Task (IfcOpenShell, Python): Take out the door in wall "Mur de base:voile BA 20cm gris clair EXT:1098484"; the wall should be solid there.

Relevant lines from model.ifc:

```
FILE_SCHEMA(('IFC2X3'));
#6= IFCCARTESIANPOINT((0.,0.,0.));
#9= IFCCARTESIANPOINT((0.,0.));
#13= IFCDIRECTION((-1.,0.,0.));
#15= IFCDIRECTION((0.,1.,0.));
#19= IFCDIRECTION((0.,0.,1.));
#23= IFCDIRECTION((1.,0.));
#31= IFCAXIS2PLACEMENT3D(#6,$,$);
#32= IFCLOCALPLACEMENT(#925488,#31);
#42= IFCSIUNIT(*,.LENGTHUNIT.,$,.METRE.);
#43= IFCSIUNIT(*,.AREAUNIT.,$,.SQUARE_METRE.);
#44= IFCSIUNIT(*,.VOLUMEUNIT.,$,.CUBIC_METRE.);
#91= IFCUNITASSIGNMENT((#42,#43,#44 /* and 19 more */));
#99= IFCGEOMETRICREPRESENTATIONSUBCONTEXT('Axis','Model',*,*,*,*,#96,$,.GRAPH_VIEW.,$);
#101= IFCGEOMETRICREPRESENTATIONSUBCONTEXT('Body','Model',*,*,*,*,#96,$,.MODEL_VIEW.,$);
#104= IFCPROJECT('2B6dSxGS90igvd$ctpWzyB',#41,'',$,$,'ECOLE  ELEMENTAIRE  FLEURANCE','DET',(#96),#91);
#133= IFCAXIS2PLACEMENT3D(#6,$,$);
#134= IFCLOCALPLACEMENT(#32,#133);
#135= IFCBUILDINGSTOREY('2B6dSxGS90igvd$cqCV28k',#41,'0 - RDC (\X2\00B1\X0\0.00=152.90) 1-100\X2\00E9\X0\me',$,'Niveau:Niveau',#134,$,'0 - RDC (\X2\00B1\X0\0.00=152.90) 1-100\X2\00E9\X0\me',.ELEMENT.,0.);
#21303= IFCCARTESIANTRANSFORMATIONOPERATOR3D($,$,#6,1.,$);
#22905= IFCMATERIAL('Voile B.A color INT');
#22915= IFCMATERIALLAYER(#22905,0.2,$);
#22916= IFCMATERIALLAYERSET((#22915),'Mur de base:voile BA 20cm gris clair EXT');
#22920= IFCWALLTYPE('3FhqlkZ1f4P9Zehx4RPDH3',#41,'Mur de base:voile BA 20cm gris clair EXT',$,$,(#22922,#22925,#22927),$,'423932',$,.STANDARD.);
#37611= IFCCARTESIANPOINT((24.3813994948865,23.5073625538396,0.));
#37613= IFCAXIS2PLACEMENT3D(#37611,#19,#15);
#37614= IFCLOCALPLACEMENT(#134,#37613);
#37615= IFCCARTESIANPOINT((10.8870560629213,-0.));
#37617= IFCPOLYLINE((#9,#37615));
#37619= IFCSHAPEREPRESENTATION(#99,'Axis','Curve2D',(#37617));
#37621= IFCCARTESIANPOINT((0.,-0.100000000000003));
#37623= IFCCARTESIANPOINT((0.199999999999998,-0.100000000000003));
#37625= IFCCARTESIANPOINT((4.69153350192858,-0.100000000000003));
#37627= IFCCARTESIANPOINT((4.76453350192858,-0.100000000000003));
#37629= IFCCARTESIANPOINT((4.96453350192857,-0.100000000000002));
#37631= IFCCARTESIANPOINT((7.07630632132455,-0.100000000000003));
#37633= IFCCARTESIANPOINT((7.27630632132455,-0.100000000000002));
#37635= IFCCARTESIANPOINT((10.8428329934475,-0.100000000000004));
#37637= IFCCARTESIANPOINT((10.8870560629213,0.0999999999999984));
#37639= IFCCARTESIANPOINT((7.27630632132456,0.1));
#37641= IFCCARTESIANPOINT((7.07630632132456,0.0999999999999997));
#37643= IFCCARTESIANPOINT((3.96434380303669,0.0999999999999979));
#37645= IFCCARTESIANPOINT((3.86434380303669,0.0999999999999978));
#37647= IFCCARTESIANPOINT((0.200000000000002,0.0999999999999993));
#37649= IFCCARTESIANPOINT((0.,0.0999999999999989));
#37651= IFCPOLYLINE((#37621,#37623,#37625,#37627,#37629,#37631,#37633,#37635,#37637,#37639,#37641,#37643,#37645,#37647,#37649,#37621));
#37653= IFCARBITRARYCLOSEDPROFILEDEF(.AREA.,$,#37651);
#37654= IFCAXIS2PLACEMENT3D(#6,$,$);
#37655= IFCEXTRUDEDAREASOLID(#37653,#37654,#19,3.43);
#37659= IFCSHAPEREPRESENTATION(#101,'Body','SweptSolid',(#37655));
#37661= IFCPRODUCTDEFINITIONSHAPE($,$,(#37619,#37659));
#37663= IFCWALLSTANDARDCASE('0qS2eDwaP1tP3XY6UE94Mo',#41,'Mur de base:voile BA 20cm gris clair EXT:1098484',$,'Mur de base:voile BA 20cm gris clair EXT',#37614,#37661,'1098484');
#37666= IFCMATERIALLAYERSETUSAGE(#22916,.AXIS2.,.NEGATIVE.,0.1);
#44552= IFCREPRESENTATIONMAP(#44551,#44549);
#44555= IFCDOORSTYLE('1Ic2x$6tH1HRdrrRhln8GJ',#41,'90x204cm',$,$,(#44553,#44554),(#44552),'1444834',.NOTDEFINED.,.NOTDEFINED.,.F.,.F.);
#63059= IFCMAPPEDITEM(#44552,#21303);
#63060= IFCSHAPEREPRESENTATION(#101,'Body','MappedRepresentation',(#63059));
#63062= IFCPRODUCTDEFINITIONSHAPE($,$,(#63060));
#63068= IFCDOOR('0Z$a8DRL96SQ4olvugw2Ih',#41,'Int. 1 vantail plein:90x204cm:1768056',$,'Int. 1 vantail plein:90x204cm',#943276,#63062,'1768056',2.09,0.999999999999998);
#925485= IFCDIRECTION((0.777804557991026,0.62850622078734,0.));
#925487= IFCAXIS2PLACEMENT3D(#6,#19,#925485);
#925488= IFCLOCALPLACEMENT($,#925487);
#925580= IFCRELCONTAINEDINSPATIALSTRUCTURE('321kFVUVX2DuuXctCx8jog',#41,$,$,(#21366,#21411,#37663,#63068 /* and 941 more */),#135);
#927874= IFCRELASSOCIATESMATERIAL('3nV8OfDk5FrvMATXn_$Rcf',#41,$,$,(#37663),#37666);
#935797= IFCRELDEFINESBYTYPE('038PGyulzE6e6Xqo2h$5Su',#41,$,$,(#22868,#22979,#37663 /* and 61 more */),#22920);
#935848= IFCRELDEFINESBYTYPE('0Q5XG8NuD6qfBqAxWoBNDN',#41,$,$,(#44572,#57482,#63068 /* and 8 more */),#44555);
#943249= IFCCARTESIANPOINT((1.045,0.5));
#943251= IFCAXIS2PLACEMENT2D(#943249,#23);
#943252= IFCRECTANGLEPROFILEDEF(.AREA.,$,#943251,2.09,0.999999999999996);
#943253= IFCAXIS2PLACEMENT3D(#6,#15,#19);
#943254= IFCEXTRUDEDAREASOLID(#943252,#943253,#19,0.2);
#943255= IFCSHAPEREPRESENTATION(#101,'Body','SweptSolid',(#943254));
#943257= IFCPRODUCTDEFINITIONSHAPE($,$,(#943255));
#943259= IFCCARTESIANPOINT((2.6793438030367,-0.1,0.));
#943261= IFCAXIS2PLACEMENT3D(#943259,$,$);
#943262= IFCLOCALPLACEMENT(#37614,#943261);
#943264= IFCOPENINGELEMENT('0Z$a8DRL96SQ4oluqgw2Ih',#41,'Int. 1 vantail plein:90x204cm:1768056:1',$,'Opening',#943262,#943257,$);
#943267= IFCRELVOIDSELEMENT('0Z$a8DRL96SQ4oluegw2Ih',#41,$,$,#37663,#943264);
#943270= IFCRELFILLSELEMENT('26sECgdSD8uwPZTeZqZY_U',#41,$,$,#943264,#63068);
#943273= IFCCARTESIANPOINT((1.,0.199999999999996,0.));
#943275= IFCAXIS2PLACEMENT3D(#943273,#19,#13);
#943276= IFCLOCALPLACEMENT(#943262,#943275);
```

```python
import ifcopenshell
import ifcopenshell.api.feature
import ifcopenshell.api.root
import ifcopenshell.geom
import ifcopenshell.util.shape

model = ifcopenshell.open("model.ifc")
settings = ifcopenshell.geom.settings()


def volume(element):
    """Net volume in cubic metres, openings subtracted."""
    shape = ifcopenshell.geom.create_shape(settings, element)
    return ifcopenshell.util.shape.get_volume(shape.geometry)


door = model.by_guid("0Z$a8DRL96SQ4olvugw2Ih")
opening = door.FillsVoids[0].RelatingOpeningElement
wall = opening.VoidsElements[0].RelatingBuildingElement
before = volume(wall)

ifcopenshell.api.root.remove_product(model, product=door)
ifcopenshell.api.feature.remove_feature(model, feature=opening)

after = volume(wall)

print(f"wall volume {before:.3f} -> {after:.3f} m3")

model.write("model_rev.ifc")
```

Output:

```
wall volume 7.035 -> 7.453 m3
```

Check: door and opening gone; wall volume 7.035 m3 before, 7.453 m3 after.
